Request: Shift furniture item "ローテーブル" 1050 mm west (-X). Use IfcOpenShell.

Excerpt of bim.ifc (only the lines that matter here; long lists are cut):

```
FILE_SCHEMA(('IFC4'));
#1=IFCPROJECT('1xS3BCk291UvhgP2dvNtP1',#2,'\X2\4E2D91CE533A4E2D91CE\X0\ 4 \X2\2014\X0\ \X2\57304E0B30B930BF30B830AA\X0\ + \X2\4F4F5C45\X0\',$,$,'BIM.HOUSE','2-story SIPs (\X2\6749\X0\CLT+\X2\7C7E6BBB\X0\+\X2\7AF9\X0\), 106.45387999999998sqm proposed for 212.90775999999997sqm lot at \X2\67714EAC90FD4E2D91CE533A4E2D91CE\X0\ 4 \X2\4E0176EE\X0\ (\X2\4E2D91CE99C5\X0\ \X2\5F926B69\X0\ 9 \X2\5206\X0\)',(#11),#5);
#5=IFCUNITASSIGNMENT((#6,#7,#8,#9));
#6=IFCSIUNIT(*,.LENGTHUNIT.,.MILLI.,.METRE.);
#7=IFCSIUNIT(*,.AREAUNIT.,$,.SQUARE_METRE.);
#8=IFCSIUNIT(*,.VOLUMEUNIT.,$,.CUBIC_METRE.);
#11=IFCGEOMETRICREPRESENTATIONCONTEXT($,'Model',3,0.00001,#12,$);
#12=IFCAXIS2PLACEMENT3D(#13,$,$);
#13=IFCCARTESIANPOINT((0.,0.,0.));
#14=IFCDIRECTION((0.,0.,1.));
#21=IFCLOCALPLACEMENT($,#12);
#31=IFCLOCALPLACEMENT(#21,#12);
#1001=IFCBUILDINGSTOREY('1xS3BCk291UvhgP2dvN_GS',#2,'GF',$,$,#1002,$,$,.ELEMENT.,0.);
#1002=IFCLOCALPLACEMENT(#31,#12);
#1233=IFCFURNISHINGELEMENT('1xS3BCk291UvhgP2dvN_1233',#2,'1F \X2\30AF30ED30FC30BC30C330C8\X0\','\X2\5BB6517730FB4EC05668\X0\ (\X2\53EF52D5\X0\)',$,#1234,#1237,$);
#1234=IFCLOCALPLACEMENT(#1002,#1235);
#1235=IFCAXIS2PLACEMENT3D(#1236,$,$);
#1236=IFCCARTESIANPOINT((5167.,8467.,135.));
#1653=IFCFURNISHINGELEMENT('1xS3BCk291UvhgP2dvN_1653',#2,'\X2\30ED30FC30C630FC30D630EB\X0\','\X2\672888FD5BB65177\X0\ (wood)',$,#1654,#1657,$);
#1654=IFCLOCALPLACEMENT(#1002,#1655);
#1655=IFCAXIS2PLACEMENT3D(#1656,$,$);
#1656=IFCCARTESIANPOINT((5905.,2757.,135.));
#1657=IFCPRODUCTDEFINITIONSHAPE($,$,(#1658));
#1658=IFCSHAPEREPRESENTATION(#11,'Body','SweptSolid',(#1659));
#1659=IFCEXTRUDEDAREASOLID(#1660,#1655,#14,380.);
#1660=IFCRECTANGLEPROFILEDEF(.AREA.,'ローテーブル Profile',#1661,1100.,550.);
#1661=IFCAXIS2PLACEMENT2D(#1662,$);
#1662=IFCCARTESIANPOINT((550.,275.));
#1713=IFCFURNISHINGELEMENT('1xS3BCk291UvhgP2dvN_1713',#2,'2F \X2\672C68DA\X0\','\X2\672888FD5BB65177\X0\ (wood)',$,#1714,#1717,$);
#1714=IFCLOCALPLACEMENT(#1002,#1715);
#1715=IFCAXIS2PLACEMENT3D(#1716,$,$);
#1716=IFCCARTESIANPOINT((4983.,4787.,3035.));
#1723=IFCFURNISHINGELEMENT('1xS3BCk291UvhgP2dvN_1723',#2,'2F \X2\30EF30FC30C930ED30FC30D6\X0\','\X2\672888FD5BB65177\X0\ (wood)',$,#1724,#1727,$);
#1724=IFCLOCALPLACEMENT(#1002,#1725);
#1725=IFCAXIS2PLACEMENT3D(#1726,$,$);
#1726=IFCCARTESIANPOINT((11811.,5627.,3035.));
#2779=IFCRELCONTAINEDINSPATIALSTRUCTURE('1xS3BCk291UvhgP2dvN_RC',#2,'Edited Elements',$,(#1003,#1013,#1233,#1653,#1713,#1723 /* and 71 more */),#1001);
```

```python
import ifcopenshell
import ifcopenshell.api.geometry
import ifcopenshell.util.placement
import ifcopenshell.util.unit

model = ifcopenshell.open("bim.ifc")
unit_scale = ifcopenshell.util.unit.calculate_unit_scale(model)

item = model.by_guid("1xS3BCk291UvhgP2dvN_1653")
matrix = ifcopenshell.util.placement.get_local_placement(item.ObjectPlacement)
matrix[0, 3] -= 1.05 / unit_scale
ifcopenshell.api.geometry.edit_object_placement(model, product=item, matrix=matrix, is_si=False)

print(ifcopenshell.util.placement.get_local_placement(item.ObjectPlacement).round(3) + 0.0)

model.write("bim_rev.ifc")
```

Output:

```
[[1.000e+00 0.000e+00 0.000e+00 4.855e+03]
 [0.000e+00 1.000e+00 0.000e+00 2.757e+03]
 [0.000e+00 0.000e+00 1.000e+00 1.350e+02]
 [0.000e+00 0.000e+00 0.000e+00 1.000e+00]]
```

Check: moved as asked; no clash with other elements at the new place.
